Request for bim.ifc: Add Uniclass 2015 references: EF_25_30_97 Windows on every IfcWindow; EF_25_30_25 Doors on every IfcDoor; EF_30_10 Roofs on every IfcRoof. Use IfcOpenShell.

First a look at what the model holds.

```python
import ifcopenshell

model = ifcopenshell.open("bim.ifc")
print(model.schema)
print("classifications:", [c.Name for c in model.by_type("IfcClassification")])
for ifc_class in ("IfcDoor", "IfcRoof", "IfcStair", "IfcWall", "IfcWindow"):
    print(ifc_class, len(model.by_type(ifc_class)))
```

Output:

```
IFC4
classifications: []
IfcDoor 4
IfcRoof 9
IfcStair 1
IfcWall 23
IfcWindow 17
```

```python
import ifcopenshell
import ifcopenshell.api.classification

model = ifcopenshell.open("bim.ifc")

system = ifcopenshell.api.classification.add_classification(model, classification="Uniclass 2015")

codes = {
    "IfcWindow": ("EF_25_30_97", "Windows"),
    "IfcDoor": ("EF_25_30_25", "Doors"),
    "IfcRoof": ("EF_30_10", "Roofs"),
}
for ifc_class, (code, name) in codes.items():
    products = model.by_type(ifc_class)
    ifcopenshell.api.classification.add_reference(
        model, products=products, classification=system, identification=code, name=name
    )
    print(code, len(products))

model.write("bim-out.ifc")
```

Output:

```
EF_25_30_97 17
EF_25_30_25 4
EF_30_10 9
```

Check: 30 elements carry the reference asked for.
